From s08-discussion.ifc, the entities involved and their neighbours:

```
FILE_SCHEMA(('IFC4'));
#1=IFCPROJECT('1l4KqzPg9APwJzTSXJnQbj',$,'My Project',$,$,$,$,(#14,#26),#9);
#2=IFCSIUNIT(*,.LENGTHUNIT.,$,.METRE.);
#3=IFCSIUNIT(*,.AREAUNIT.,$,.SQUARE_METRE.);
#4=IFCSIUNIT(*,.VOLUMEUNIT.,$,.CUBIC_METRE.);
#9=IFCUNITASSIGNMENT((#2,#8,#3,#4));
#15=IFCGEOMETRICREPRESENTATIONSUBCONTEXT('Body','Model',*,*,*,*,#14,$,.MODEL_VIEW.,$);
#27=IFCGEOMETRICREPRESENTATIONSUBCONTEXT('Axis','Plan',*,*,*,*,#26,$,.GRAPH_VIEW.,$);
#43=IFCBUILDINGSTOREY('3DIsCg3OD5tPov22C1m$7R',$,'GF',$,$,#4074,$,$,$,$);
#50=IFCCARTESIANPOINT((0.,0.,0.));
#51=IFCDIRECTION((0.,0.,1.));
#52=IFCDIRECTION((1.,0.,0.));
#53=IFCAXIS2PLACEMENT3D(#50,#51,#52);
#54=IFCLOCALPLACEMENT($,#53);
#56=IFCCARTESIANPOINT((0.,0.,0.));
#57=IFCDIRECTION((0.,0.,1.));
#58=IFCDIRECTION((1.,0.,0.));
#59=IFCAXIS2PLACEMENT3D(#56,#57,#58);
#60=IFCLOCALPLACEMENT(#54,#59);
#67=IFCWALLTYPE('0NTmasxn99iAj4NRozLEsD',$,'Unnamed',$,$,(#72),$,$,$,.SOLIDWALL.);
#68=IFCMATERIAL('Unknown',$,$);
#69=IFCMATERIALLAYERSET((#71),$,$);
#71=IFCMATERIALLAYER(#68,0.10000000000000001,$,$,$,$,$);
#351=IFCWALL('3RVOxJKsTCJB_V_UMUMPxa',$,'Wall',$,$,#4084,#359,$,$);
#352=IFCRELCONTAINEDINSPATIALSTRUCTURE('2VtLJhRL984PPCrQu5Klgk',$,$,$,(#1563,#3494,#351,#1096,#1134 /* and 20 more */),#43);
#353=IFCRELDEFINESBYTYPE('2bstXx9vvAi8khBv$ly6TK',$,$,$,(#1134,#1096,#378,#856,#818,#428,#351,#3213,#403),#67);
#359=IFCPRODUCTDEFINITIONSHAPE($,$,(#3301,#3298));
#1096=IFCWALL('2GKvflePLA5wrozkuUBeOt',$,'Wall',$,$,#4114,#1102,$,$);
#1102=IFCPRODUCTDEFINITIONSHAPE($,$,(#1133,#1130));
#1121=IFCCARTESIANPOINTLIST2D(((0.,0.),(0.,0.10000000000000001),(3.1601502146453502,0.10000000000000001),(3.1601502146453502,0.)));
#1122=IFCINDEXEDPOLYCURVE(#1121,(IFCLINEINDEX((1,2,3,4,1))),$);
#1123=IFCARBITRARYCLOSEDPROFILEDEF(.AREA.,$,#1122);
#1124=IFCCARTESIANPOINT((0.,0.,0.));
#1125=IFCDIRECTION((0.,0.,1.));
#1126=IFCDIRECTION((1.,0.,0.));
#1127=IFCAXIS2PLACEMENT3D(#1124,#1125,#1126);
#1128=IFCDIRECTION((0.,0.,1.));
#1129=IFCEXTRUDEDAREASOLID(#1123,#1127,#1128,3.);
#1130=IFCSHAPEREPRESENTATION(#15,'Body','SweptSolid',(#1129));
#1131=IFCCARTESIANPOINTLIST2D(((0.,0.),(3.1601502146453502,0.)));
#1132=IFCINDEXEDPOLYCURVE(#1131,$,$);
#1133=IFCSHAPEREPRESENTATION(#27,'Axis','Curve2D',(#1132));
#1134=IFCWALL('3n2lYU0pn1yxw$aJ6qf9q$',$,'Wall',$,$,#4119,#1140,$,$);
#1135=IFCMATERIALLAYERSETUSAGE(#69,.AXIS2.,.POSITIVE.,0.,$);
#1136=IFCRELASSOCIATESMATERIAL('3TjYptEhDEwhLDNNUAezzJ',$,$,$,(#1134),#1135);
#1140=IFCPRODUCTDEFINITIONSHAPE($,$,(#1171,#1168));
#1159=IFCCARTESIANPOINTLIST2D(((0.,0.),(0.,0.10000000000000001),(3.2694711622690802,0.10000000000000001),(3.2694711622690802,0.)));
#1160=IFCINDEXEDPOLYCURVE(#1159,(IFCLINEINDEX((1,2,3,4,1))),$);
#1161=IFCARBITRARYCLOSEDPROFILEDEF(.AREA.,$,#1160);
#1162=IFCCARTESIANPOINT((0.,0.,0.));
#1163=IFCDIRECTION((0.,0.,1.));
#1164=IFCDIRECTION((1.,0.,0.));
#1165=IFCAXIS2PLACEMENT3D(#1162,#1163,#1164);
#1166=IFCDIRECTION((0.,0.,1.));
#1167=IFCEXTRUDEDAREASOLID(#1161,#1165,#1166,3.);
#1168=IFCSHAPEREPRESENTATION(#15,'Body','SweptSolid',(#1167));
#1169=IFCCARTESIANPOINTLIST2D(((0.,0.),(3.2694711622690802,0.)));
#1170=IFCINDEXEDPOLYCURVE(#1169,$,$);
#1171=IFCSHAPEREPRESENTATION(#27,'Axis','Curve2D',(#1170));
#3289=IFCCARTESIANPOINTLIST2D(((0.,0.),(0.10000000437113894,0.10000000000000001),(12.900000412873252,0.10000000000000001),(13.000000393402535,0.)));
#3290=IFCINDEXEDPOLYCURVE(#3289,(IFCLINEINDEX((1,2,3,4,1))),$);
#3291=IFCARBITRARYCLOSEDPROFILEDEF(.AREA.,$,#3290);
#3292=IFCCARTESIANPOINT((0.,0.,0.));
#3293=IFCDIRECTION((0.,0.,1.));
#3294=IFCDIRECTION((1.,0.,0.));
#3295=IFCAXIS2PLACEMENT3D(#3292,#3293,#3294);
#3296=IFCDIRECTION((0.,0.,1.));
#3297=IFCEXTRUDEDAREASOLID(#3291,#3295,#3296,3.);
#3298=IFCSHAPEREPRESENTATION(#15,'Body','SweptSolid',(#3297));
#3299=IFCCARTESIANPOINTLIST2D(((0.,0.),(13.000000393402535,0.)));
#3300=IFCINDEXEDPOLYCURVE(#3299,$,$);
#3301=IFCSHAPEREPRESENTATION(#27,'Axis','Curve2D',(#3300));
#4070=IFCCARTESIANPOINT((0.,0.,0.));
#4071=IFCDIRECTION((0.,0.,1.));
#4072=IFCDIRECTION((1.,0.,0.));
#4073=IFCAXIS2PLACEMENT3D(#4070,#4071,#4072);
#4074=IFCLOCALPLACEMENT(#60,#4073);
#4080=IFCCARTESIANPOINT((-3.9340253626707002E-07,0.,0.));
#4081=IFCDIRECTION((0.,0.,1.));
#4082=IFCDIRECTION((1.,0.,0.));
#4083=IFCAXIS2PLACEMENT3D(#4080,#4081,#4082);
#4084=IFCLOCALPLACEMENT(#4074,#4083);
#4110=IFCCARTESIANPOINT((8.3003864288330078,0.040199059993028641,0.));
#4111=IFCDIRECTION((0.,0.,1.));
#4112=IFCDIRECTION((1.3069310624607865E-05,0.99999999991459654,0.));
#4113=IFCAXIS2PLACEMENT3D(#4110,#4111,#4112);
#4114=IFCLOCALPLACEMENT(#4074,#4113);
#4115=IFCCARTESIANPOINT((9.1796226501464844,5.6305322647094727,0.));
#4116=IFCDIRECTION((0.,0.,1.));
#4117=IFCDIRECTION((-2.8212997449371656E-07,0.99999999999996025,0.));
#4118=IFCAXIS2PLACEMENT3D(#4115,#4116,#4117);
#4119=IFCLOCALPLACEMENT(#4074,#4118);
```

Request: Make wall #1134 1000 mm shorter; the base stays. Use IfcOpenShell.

```python
import ifcopenshell
import ifcopenshell.geom
import ifcopenshell.util.representation
import ifcopenshell.util.shape

model = ifcopenshell.open("s08-discussion.ifc")
settings = ifcopenshell.geom.settings()


def volume(element):
    """Net volume in cubic metres, openings subtracted."""
    shape = ifcopenshell.geom.create_shape(settings, element)
    return ifcopenshell.util.shape.get_volume(shape.geometry)


wall = model.by_id(1134)
before = volume(wall)

body = ifcopenshell.util.representation.get_representation(wall, "Model", "Body")
solid = body.Items[0]
old_height = solid.Depth
solid.Depth -= 1.0
after = volume(wall)

print(f"height {old_height:g} -> {solid.Depth:g}, volume {before:.3f} -> {after:.3f} m3")

model.write("s08-discussion_edited.ifc")
```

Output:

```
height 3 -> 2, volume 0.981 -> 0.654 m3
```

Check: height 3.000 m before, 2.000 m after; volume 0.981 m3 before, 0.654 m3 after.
